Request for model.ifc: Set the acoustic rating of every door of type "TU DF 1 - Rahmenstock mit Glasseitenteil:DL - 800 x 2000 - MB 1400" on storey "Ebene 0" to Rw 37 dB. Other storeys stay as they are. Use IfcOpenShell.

First a look at what the model holds.

```python
import ifcopenshell
import ifcopenshell.util.element

model = ifcopenshell.open("model.ifc")
print(model.schema)
storey = next(s for s in model.by_type("IfcBuildingStorey") if s.Name == "Ebene 0")
doors = [e for e in ifcopenshell.util.element.get_decomposition(storey) if e.is_a("IfcDoor")]
seen = {}
for e in doors:
    element_type = ifcopenshell.util.element.get_type(e)
    key = (element_type.Name if element_type != e and element_type else None, ifcopenshell.util.element.get_pset(e, "Pset_DoorCommon", "AcousticRating"))
    seen[key] = seen.get(key, 0) + 1
for (name, value), count in sorted(seen.items(), key=str):
    print(count, "x", name, "|", value)
```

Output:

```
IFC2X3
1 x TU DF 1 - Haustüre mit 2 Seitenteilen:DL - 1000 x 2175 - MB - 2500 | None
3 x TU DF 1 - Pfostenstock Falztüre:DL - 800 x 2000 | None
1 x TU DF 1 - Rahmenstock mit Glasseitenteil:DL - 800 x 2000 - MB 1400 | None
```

```python
import ifcopenshell
import ifcopenshell.api.pset
import ifcopenshell.util.element

model = ifcopenshell.open("model.ifc")

storey = next(s for s in model.by_type("IfcBuildingStorey") if s.Name == "Ebene 0")
doors = [e for e in ifcopenshell.util.element.get_decomposition(storey) if e.is_a("IfcDoor")]

count = 0
for e in doors:
    element_type = ifcopenshell.util.element.get_type(e)
    if element_type in (None, e) or element_type.Name != "TU DF 1 - Rahmenstock mit Glasseitenteil:DL - 800 x 2000 - MB 1400":
        continue
    # add_pset returns the element's existing set when there is one.
    pset = ifcopenshell.api.pset.add_pset(model, product=e, name="Pset_DoorCommon")
    ifcopenshell.api.pset.edit_pset(model, pset=pset, properties={"AcousticRating": "Rw 37 dB"})
    count += 1

print(count, "doors updated")

model.write("model-out.ifc")
```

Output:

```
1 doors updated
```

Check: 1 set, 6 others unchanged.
